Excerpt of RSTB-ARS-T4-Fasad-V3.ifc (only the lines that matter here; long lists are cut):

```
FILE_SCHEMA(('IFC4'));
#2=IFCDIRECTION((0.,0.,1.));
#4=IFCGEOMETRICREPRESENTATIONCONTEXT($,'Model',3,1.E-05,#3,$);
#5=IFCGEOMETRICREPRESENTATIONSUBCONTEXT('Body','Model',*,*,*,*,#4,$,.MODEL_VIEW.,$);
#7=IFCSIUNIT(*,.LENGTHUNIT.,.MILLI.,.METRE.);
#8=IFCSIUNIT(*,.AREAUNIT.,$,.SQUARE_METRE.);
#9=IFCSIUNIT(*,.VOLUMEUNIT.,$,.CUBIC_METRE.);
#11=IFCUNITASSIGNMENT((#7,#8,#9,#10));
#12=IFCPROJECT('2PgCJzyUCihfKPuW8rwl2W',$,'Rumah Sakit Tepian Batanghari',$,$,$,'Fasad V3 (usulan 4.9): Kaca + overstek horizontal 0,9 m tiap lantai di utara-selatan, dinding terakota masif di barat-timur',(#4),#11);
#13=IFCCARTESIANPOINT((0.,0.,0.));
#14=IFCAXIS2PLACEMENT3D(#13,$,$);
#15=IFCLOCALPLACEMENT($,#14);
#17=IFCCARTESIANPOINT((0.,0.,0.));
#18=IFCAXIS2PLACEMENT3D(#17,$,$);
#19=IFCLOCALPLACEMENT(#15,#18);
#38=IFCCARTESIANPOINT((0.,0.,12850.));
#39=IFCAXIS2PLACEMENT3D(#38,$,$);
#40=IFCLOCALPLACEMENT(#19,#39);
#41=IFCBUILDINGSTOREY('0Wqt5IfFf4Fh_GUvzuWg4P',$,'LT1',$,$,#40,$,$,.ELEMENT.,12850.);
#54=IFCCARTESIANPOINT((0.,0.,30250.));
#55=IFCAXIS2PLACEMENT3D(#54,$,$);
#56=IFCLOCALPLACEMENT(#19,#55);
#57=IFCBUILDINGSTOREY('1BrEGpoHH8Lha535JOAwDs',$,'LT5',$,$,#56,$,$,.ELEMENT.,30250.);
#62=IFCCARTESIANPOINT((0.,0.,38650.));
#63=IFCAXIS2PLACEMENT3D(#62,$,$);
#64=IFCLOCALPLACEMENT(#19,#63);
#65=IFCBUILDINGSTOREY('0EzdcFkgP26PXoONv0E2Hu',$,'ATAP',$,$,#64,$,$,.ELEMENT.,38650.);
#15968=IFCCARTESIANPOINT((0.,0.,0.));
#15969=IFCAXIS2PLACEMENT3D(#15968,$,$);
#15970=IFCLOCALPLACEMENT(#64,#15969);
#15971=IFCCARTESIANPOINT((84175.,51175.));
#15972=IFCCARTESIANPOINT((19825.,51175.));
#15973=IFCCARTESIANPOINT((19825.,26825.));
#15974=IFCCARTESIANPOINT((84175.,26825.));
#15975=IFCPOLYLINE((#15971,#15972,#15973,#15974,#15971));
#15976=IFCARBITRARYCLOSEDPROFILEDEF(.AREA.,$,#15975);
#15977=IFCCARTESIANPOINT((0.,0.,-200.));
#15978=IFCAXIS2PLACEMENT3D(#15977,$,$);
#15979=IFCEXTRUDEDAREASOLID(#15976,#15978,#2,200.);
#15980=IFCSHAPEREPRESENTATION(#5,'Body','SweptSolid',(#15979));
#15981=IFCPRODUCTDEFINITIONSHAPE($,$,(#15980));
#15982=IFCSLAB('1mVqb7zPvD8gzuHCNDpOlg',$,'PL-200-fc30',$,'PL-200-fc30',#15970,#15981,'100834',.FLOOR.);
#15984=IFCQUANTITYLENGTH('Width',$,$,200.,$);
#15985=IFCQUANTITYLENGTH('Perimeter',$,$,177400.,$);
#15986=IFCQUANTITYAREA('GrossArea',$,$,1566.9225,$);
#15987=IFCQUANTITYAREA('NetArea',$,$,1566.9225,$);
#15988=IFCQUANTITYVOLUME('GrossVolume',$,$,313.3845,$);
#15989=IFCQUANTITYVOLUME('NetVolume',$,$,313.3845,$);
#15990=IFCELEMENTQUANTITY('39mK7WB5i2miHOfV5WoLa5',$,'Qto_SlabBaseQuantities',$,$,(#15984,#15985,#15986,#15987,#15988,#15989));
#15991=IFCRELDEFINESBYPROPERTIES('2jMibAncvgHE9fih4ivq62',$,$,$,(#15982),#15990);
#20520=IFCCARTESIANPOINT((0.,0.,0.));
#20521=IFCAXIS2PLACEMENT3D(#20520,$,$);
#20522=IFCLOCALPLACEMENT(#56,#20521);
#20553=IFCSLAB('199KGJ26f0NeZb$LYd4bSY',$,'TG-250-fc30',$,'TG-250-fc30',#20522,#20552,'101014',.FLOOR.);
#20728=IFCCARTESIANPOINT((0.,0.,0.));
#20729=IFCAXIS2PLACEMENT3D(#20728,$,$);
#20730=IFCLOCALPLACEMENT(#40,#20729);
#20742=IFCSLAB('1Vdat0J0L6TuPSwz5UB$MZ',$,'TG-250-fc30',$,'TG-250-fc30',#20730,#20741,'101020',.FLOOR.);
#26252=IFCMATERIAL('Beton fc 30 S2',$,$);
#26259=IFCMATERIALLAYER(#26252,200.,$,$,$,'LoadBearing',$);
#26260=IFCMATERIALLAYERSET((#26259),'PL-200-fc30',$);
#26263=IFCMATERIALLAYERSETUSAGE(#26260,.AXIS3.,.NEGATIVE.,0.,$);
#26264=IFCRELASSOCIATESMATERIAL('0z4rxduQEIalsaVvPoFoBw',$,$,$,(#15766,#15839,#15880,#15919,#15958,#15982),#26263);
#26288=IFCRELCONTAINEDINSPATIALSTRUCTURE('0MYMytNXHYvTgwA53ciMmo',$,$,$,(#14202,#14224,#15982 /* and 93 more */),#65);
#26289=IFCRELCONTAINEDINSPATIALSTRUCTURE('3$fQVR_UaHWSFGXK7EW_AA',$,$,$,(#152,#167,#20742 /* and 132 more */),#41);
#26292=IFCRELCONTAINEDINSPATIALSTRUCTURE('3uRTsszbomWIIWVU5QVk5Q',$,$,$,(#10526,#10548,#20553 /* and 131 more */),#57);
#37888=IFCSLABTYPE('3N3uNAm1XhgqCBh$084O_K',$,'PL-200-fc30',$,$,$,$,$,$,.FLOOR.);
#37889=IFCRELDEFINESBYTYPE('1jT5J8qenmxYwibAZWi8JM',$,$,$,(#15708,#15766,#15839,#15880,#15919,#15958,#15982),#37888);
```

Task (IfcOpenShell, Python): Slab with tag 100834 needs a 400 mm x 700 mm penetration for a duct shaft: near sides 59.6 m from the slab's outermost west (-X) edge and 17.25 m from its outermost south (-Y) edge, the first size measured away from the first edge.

```python
import numpy as np
import ifcopenshell
import ifcopenshell.api.feature
import ifcopenshell.api.geometry
import ifcopenshell.api.pset
import ifcopenshell.api.root
import ifcopenshell.geom
import ifcopenshell.util.element
import ifcopenshell.util.placement
import ifcopenshell.util.representation
import ifcopenshell.util.shape
import ifcopenshell.util.unit

model = ifcopenshell.open("RSTB-ARS-T4-Fasad-V3.ifc")
unit_scale = ifcopenshell.util.unit.calculate_unit_scale(model)
area_scale = ifcopenshell.util.unit.calculate_unit_scale(model, "AREAUNIT")
volume_scale = ifcopenshell.util.unit.calculate_unit_scale(model, "VOLUMEUNIT")
settings = ifcopenshell.geom.settings()


def volume(element):
    """Net volume in cubic metres, openings subtracted."""
    shape = ifcopenshell.geom.create_shape(settings, element)
    return ifcopenshell.util.shape.get_volume(shape.geometry)


slab = model.by_guid("1mVqb7zPvD8gzuHCNDpOlg")
before = volume(slab)

# Extent in the slab's own axes, in metres. The edges named are its -X and -Y sides.
slab_shape = ifcopenshell.geom.create_shape(settings, slab)
vertices = ifcopenshell.util.shape.get_vertices(slab_shape.geometry)
x_min, y_min, bottom = vertices.min(axis=0)
top = vertices[:, 2].max()

opening = ifcopenshell.api.root.create_entity(model, ifc_class="IfcOpeningElement", name="Duct shaft opening", predefined_type="OPENING")
context = ifcopenshell.util.representation.get_context(model, "Model", "Body", "MODEL_VIEW")
width, depth = 0.4, 0.7
outline = [(0.0, 0.0), (width, 0.0), (width, depth), (0.0, depth), (0.0, 0.0)]
# Overshoot both faces by 50 mm so the cut is clean.
shape = ifcopenshell.api.geometry.add_slab_representation(
    model, context=context, depth=top - bottom + 0.1, polyline=outline
)
ifcopenshell.api.geometry.assign_representation(model, product=opening, representation=shape)

matrix = ifcopenshell.util.placement.get_local_placement(slab.ObjectPlacement)
matrix[:, 3] = matrix @ np.append(np.array([x_min + 59.6, y_min + 17.25, bottom - 0.05]) / unit_scale, 1.0)
ifcopenshell.api.geometry.edit_object_placement(model, product=opening, matrix=matrix, is_si=False)
ifcopenshell.api.feature.add_feature(model, feature=opening, element=slab)

after = volume(slab)

# Update the slab's stored quantities.
qto = model.by_id(ifcopenshell.util.element.get_pset(slab, "Qto_SlabBaseQuantities", should_inherit=False)["id"])
ifcopenshell.api.pset.edit_qto(model, qto=qto, properties={
    "NetArea": after / (top - bottom) / area_scale,
    "NetVolume": after / volume_scale,
})

print(f"slab volume {before:.3f} -> {after:.3f} m3")

model.write("RSTB-ARS-T4-Fasad-V3_updated.ifc")
```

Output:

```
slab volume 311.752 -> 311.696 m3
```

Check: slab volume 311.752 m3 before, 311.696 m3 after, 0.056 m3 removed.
